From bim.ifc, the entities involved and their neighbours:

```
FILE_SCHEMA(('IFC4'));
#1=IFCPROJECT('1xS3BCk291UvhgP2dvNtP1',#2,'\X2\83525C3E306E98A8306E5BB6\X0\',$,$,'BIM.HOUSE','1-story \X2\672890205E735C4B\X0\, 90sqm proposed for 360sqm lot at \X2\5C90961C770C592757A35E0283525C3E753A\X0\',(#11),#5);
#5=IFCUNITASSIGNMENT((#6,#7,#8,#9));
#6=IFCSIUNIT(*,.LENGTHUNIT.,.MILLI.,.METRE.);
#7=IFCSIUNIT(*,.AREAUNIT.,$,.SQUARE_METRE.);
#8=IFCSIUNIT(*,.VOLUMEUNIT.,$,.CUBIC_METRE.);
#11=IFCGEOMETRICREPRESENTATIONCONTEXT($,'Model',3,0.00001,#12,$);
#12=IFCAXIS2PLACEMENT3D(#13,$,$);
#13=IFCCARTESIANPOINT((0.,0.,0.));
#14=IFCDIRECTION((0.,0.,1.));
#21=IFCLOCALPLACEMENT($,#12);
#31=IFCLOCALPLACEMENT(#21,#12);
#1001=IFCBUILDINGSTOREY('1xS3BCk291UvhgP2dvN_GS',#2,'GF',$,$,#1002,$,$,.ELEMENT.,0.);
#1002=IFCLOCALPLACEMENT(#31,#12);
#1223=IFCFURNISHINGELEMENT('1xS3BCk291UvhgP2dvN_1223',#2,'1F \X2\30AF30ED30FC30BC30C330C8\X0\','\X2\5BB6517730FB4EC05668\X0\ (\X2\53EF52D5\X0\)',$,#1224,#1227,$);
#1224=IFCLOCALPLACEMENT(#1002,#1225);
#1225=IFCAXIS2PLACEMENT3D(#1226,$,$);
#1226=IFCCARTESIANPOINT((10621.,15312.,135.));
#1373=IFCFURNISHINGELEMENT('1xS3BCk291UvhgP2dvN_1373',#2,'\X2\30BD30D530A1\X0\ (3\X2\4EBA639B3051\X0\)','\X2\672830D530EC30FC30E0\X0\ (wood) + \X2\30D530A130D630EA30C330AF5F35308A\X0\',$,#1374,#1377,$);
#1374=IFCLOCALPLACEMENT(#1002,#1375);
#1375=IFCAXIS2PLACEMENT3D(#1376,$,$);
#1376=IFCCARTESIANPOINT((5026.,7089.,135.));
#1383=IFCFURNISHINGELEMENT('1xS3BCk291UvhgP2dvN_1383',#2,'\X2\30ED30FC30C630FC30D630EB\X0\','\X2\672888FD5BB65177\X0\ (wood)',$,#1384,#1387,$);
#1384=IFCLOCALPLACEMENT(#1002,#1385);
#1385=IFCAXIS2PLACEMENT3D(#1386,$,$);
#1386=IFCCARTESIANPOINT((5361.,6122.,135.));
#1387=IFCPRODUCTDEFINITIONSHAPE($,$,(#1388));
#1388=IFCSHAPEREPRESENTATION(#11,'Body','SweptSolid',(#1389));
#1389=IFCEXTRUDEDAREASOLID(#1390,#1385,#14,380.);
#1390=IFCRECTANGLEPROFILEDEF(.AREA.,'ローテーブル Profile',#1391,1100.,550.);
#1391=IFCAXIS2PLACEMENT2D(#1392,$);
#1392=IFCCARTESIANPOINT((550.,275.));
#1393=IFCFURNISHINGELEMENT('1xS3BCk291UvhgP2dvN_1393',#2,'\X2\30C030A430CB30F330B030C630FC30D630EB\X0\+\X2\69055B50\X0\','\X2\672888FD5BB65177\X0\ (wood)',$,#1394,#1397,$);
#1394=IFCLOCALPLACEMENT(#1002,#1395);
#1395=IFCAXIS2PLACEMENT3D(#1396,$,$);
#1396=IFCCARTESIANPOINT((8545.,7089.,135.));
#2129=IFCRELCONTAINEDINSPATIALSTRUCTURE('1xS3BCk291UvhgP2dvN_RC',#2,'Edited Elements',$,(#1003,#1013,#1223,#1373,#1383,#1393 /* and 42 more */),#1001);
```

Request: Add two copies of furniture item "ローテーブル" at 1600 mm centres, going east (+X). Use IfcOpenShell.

```python
import numpy as np
import ifcopenshell
import ifcopenshell.api.geometry
import ifcopenshell.api.root
import ifcopenshell.util.element
import ifcopenshell.util.placement

model = ifcopenshell.open("bim.ifc")


def reuse_history(source, copy):
    """copy_class also copies each property set's owner history, people and application; keep the originals."""
    for rel in copy.IsDefinedBy:
        if rel.is_a("IfcRelDefinesByProperties") and (history := rel.RelatingPropertyDefinition.OwnerHistory):
            rel.RelatingPropertyDefinition.OwnerHistory = source.OwnerHistory
            ifcopenshell.util.element.remove_deep2(model, history)


source = model.by_guid("1xS3BCk291UvhgP2dvN_1383")
base = ifcopenshell.util.placement.get_local_placement(source.ObjectPlacement)
step = np.array([1.0, 0.0, 0.0]) * 1600.0

for i in range(1, 3):
    copy = ifcopenshell.api.root.copy_class(model, product=source)
    copy.Representation = ifcopenshell.util.element.copy_deep(
        model, source.Representation, exclude=["IfcGeometricRepresentationContext", "IfcRepresentationMap"]
    )
    reuse_history(source, copy)
    matrix = base.copy()
    matrix[:3, 3] += i * step
    print("added at", matrix[:3, 3].round(3) + 0.0)
    ifcopenshell.api.geometry.edit_object_placement(model, product=copy, matrix=matrix, is_si=False)

model.write("bim_rev.ifc")
```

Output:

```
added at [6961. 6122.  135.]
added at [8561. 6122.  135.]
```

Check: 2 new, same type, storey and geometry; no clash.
